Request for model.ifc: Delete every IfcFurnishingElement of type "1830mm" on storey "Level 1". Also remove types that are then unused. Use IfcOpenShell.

First a look at what the model holds.

```python
import ifcopenshell
import ifcopenshell.util.element

model = ifcopenshell.open("model.ifc")
print(model.schema)
storey = next(s for s in model.by_type("IfcBuildingStorey") if s.Name == "Level 1")
furniture = [e for e in ifcopenshell.util.element.get_decomposition(storey) if e.is_a("IfcFurnishingElement")]
seen = {}
for e in furniture:
    element_type = ifcopenshell.util.element.get_type(e)
    name = element_type.Name if element_type not in (None, e) else None
    seen[name] = seen.get(name, 0) + 1
for name, count in sorted(seen.items(), key=str):
    print(count, "x", name)
```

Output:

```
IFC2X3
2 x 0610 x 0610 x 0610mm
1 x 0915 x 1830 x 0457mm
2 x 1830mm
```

```python
import ifcopenshell
import ifcopenshell.api.root
import ifcopenshell.util.element

model = ifcopenshell.open("model.ifc")

storey = next(s for s in model.by_type("IfcBuildingStorey") if s.Name == "Level 1")
furniture = [e for e in ifcopenshell.util.element.get_decomposition(storey) if e.is_a("IfcFurnishingElement")]
targets = [e for e in furniture if (t := ifcopenshell.util.element.get_type(e)) not in (None, e) and t.Name == "1830mm"]
types = {ifcopenshell.util.element.get_type(e) for e in targets} - {None, *targets}

for e in targets:
    ifcopenshell.api.root.remove_product(model, product=e)
print(len(targets), "removed")

unused = [t for t in types if not ifcopenshell.util.element.get_types(t)]
for t in unused:
    ifcopenshell.api.root.remove_product(model, product=t)
print(len(unused), "unused types removed")

model.write("model_edited.ifc")
```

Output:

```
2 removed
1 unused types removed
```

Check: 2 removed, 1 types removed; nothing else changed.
